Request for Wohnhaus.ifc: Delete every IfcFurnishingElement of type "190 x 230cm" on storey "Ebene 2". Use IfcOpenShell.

First a look at what the model holds.

```python
import ifcopenshell
import ifcopenshell.util.element

model = ifcopenshell.open("Wohnhaus.ifc")
print(model.schema)
storey = next(s for s in model.by_type("IfcBuildingStorey") if s.Name == "Ebene 2")
furniture = [e for e in ifcopenshell.util.element.get_decomposition(storey) if e.is_a("IfcFurnishingElement")]
seen = {}
for e in furniture:
    element_type = ifcopenshell.util.element.get_type(e)
    name = element_type.Name if element_type not in (None, e) else None
    seen[name] = seen.get(name, 0) + 1
for name, count in sorted(seen.items(), key=str):
    print(count, "x", name)
```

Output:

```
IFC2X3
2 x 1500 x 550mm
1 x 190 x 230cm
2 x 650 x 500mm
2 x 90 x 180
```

```python
import ifcopenshell
import ifcopenshell.api.root
import ifcopenshell.util.element

model = ifcopenshell.open("Wohnhaus.ifc")

storey = next(s for s in model.by_type("IfcBuildingStorey") if s.Name == "Ebene 2")
furniture = [e for e in ifcopenshell.util.element.get_decomposition(storey) if e.is_a("IfcFurnishingElement")]
targets = [e for e in furniture if (t := ifcopenshell.util.element.get_type(e)) not in (None, e) and t.Name == "190 x 230cm"]

for e in targets:
    ifcopenshell.api.root.remove_product(model, product=e)
print(len(targets), "removed")

model.write("Wohnhaus_updated.ifc")
```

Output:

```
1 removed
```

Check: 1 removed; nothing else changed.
